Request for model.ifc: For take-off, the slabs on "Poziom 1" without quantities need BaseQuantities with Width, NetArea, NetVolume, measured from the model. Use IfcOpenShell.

First a look at what the model holds.

```python
import ifcopenshell
import ifcopenshell.util.element
import ifcopenshell.util.unit

model = ifcopenshell.open("model.ifc")
print(model.schema)
for unit_type in ("LENGTHUNIT", "AREAUNIT", "VOLUMEUNIT"):
    print(unit_type, ifcopenshell.util.unit.calculate_unit_scale(model, unit_type))
storey = next(s for s in model.by_type("IfcBuildingStorey") if s.Name == "Poziom 1")
slabs = [e for e in ifcopenshell.util.element.get_decomposition(storey) if e.is_a("IfcSlab")]
for e in sorted(slabs, key=lambda e: e.id()):
    print(e.id(), e.is_a(), e.Name, list(ifcopenshell.util.element.get_psets(e, qtos_only=True)), sep=" | ")
```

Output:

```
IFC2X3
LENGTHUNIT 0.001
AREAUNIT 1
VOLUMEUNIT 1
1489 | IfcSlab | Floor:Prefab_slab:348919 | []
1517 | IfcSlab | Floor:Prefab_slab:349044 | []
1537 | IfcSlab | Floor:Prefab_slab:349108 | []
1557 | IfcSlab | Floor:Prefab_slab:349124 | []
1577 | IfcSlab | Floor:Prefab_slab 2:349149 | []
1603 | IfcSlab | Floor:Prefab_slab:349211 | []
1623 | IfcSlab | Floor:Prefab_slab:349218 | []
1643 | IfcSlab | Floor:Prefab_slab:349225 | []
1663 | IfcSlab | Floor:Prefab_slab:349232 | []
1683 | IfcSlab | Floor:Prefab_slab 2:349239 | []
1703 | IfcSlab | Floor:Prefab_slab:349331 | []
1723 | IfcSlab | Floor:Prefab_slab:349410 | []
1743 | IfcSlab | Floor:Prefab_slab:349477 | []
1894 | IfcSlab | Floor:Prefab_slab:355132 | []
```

```python
import ifcopenshell
import ifcopenshell.api.pset
import ifcopenshell.geom
import ifcopenshell.util.element
import ifcopenshell.util.shape
import ifcopenshell.util.unit

model = ifcopenshell.open("model.ifc")
unit_scale = ifcopenshell.util.unit.calculate_unit_scale(model)
area_scale = ifcopenshell.util.unit.calculate_unit_scale(model, "AREAUNIT")
volume_scale = ifcopenshell.util.unit.calculate_unit_scale(model, "VOLUMEUNIT")
settings = ifcopenshell.geom.settings()

storey = next(s for s in model.by_type("IfcBuildingStorey") if s.Name == "Poziom 1")
slabs = [e for e in ifcopenshell.util.element.get_decomposition(storey) if e.is_a("IfcSlab")]

for e in sorted(slabs, key=lambda e: e.id()):
    if ifcopenshell.util.element.get_psets(e, qtos_only=True, should_inherit=False):
        continue
    # Geometry comes back in metres, in the element's own axes.
    shape = ifcopenshell.geom.create_shape(settings, e)
    values = {
        "Width": ifcopenshell.util.shape.get_z(shape.geometry) / unit_scale,
        "NetArea": ifcopenshell.util.shape.get_footprint_area(shape.geometry) / area_scale,
        "NetVolume": ifcopenshell.util.shape.get_volume(shape.geometry) / volume_scale,
    }
    qto = ifcopenshell.api.pset.add_qto(model, product=e, name="BaseQuantities")
    ifcopenshell.api.pset.edit_qto(model, qto=qto, properties=values)
    print(e.id(), {k: round(v, 3) for k, v in values.items()})

model.write("model_updated.ifc")
```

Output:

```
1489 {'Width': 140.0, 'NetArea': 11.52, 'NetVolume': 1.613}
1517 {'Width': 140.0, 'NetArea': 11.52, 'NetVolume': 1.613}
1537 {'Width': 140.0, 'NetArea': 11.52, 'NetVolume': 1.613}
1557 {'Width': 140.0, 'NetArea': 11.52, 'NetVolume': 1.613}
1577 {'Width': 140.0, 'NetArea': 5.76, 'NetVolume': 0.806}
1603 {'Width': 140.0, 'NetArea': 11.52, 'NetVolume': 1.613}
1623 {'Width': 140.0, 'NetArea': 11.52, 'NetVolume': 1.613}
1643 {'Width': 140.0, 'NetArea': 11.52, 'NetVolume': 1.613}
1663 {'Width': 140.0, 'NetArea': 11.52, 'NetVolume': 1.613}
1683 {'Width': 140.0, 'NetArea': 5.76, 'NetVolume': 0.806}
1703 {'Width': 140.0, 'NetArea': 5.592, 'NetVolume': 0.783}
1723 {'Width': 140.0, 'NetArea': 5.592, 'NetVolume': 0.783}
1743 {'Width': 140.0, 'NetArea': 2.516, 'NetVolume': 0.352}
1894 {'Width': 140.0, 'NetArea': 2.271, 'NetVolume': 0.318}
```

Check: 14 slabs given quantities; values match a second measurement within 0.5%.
